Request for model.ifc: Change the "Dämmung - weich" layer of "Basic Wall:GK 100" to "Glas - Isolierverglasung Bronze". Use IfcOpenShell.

First a look at what the model holds.

```python
import ifcopenshell
import ifcopenshell.util.element

model = ifcopenshell.open("model.ifc")
print(model.schema)
for layer_set in model.by_type("IfcMaterialLayerSet"):
    if layer_set.LayerSetName == "Basic Wall:GK 100":
        for layer in layer_set.MaterialLayers:
            print(layer.id(), layer.Material and layer.Material.Name, layer.LayerThickness, sep=" | ")
        print(len(ifcopenshell.util.element.get_elements_by_material(model, layer_set)), "elements and types use it")
print(sorted(m.Name for m in model.by_type("IfcMaterial") if m.Name)[:60])
```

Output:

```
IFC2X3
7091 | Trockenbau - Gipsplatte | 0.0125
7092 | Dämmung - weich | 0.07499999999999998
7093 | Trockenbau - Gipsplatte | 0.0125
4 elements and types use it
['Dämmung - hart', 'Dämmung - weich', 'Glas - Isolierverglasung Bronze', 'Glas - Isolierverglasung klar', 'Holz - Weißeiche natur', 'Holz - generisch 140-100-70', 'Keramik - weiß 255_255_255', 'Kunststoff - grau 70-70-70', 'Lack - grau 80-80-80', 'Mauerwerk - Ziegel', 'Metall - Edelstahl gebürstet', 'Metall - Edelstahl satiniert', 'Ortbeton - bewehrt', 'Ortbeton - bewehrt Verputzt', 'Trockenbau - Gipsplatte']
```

```python
import ifcopenshell
import ifcopenshell.api.material

model = ifcopenshell.open("model.ifc")

layer_set = next(s for s in model.by_type("IfcMaterialLayerSet") if s.LayerSetName == "Basic Wall:GK 100")
layer = next(l for l in layer_set.MaterialLayers if l.Material and l.Material.Name == "Dämmung - weich")
material = next(m for m in model.by_type("IfcMaterial") if m.Name == "Glas - Isolierverglasung Bronze")

# Point this one layer at the other material; renaming the old one would change it everywhere.
ifcopenshell.api.material.edit_layer(model, layer=layer, attributes={}, material=material)

print([l.Material.Name if l.Material else None for l in layer_set.MaterialLayers])

model.write("model_edited.ifc")
```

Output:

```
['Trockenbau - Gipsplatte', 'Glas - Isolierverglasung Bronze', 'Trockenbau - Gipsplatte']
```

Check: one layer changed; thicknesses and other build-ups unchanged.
